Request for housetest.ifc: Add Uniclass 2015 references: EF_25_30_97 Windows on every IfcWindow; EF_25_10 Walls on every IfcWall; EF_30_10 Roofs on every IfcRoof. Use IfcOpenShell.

First a look at what the model holds.

```python
import ifcopenshell

model = ifcopenshell.open("housetest.ifc")
print(model.schema)
print("classifications:", [c.Name for c in model.by_type("IfcClassification")])
for ifc_class in ("IfcDoor", "IfcRoof", "IfcStair", "IfcWall", "IfcWindow"):
    print(ifc_class, len(model.by_type(ifc_class)))
```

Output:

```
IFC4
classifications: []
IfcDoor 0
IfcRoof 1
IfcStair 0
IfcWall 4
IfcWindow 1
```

```python
import ifcopenshell
import ifcopenshell.api.classification

model = ifcopenshell.open("housetest.ifc")

system = ifcopenshell.api.classification.add_classification(model, classification="Uniclass 2015")

codes = {
    "IfcWindow": ("EF_25_30_97", "Windows"),
    "IfcWall": ("EF_25_10", "Walls"),
    "IfcRoof": ("EF_30_10", "Roofs"),
}
for ifc_class, (code, name) in codes.items():
    products = model.by_type(ifc_class)
    ifcopenshell.api.classification.add_reference(
        model, products=products, classification=system, identification=code, name=name
    )
    print(code, len(products))

model.write("housetest_edited.ifc")
```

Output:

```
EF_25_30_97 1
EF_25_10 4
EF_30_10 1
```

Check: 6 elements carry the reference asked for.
